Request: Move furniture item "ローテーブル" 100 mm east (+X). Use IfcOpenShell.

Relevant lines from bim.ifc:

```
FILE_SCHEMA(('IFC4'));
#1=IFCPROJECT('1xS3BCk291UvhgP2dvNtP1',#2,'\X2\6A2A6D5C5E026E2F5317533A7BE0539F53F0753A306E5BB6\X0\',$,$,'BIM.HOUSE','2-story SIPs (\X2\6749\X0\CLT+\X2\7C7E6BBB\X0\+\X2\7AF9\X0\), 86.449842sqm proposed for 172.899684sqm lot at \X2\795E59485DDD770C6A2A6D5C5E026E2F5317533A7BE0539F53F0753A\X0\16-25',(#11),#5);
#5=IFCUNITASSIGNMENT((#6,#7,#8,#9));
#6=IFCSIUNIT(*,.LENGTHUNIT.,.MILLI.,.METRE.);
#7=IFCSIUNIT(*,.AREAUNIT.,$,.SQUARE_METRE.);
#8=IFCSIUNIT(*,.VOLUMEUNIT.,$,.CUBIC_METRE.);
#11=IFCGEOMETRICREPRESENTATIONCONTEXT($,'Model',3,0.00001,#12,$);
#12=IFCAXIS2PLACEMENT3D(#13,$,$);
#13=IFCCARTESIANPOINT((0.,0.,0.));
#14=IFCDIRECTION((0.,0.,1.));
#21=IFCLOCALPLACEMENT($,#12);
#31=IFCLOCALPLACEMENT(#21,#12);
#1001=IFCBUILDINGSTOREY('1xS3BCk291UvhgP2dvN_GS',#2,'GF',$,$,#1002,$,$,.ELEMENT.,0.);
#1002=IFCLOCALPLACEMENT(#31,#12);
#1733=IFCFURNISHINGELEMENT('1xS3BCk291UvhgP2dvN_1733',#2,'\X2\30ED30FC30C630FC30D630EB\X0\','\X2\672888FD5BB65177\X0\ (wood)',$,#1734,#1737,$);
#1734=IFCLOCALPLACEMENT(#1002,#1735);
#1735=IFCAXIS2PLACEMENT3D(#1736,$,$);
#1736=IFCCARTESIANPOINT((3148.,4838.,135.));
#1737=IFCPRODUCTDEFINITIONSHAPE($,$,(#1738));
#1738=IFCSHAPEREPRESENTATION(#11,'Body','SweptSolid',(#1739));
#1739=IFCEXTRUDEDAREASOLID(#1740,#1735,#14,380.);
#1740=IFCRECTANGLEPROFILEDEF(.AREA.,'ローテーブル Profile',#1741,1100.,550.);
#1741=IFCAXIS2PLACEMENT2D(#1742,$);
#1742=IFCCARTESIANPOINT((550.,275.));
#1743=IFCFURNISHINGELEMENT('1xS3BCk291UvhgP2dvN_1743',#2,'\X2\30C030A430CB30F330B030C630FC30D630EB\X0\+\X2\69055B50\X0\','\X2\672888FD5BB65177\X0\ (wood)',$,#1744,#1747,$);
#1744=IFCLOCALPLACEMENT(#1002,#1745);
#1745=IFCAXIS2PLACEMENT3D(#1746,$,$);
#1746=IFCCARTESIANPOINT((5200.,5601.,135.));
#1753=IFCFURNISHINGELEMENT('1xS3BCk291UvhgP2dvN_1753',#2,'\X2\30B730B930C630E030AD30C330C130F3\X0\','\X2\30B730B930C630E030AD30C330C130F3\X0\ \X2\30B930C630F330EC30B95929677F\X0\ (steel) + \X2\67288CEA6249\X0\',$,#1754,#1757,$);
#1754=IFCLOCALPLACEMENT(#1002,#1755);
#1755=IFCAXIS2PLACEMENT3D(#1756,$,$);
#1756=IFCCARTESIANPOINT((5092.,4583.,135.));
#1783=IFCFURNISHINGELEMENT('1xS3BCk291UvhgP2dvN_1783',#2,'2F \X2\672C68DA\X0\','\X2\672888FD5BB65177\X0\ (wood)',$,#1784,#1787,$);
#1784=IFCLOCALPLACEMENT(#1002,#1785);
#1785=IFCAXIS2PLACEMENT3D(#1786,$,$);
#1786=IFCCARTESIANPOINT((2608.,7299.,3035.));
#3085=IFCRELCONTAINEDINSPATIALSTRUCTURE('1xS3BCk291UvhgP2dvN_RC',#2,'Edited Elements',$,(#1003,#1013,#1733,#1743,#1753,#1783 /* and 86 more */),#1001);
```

```python
import ifcopenshell
import ifcopenshell.api.geometry
import ifcopenshell.util.placement
import ifcopenshell.util.unit

model = ifcopenshell.open("bim.ifc")
unit_scale = ifcopenshell.util.unit.calculate_unit_scale(model)

item = model.by_id(1733)
matrix = ifcopenshell.util.placement.get_local_placement(item.ObjectPlacement)
matrix[0, 3] += 0.1 / unit_scale
ifcopenshell.api.geometry.edit_object_placement(model, product=item, matrix=matrix, is_si=False)

print(ifcopenshell.util.placement.get_local_placement(item.ObjectPlacement).round(3) + 0.0)

model.write("bim_updated.ifc")
```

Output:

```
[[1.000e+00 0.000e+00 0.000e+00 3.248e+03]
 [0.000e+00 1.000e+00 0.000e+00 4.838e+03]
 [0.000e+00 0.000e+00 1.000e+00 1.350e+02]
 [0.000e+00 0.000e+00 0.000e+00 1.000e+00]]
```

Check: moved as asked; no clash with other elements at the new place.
